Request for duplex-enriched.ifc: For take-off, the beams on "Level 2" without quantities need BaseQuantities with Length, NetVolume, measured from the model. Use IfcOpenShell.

First a look at what the model holds.

```python
import ifcopenshell
import ifcopenshell.util.element
import ifcopenshell.util.unit

model = ifcopenshell.open("duplex-enriched.ifc")
print(model.schema)
for unit_type in ("LENGTHUNIT", "AREAUNIT", "VOLUMEUNIT"):
    print(unit_type, ifcopenshell.util.unit.calculate_unit_scale(model, unit_type))
storey = next(s for s in model.by_type("IfcBuildingStorey") if s.Name == "Level 2")
beams = [e for e in ifcopenshell.util.element.get_decomposition(storey) if e.is_a("IfcBeam")]
for e in sorted(beams, key=lambda e: e.id()):
    print(e.id(), e.is_a(), e.Name, list(ifcopenshell.util.element.get_psets(e, qtos_only=True)), sep=" | ")
```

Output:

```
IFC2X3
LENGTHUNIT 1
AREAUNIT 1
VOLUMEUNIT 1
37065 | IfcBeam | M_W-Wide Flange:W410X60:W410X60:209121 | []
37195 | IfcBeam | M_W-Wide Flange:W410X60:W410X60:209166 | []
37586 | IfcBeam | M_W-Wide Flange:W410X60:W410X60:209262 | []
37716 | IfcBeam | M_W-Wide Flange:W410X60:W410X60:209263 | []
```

```python
import ifcopenshell
import ifcopenshell.api.pset
import ifcopenshell.geom
import ifcopenshell.util.element
import ifcopenshell.util.shape
import ifcopenshell.util.unit

model = ifcopenshell.open("duplex-enriched.ifc")
unit_scale = ifcopenshell.util.unit.calculate_unit_scale(model)
volume_scale = ifcopenshell.util.unit.calculate_unit_scale(model, "VOLUMEUNIT")
settings = ifcopenshell.geom.settings()

storey = next(s for s in model.by_type("IfcBuildingStorey") if s.Name == "Level 2")
beams = [e for e in ifcopenshell.util.element.get_decomposition(storey) if e.is_a("IfcBeam")]

for e in sorted(beams, key=lambda e: e.id()):
    if ifcopenshell.util.element.get_psets(e, qtos_only=True, should_inherit=False):
        continue
    # Geometry comes back in metres, in the element's own axes.
    shape = ifcopenshell.geom.create_shape(settings, e)
    values = {
        "Length": ifcopenshell.util.shape.get_max_xyz(shape.geometry) / unit_scale,
        "NetVolume": ifcopenshell.util.shape.get_volume(shape.geometry) / volume_scale,
    }
    qto = ifcopenshell.api.pset.add_qto(model, product=e, name="BaseQuantities")
    ifcopenshell.api.pset.edit_qto(model, qto=qto, properties=values)
    print(e.id(), {k: round(v, 3) for k, v in values.items()})

model.write("duplex-enriched_updated.ifc")
```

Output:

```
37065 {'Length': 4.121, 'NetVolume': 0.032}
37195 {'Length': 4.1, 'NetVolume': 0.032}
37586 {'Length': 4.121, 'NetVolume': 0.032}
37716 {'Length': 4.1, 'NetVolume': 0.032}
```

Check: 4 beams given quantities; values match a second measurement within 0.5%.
